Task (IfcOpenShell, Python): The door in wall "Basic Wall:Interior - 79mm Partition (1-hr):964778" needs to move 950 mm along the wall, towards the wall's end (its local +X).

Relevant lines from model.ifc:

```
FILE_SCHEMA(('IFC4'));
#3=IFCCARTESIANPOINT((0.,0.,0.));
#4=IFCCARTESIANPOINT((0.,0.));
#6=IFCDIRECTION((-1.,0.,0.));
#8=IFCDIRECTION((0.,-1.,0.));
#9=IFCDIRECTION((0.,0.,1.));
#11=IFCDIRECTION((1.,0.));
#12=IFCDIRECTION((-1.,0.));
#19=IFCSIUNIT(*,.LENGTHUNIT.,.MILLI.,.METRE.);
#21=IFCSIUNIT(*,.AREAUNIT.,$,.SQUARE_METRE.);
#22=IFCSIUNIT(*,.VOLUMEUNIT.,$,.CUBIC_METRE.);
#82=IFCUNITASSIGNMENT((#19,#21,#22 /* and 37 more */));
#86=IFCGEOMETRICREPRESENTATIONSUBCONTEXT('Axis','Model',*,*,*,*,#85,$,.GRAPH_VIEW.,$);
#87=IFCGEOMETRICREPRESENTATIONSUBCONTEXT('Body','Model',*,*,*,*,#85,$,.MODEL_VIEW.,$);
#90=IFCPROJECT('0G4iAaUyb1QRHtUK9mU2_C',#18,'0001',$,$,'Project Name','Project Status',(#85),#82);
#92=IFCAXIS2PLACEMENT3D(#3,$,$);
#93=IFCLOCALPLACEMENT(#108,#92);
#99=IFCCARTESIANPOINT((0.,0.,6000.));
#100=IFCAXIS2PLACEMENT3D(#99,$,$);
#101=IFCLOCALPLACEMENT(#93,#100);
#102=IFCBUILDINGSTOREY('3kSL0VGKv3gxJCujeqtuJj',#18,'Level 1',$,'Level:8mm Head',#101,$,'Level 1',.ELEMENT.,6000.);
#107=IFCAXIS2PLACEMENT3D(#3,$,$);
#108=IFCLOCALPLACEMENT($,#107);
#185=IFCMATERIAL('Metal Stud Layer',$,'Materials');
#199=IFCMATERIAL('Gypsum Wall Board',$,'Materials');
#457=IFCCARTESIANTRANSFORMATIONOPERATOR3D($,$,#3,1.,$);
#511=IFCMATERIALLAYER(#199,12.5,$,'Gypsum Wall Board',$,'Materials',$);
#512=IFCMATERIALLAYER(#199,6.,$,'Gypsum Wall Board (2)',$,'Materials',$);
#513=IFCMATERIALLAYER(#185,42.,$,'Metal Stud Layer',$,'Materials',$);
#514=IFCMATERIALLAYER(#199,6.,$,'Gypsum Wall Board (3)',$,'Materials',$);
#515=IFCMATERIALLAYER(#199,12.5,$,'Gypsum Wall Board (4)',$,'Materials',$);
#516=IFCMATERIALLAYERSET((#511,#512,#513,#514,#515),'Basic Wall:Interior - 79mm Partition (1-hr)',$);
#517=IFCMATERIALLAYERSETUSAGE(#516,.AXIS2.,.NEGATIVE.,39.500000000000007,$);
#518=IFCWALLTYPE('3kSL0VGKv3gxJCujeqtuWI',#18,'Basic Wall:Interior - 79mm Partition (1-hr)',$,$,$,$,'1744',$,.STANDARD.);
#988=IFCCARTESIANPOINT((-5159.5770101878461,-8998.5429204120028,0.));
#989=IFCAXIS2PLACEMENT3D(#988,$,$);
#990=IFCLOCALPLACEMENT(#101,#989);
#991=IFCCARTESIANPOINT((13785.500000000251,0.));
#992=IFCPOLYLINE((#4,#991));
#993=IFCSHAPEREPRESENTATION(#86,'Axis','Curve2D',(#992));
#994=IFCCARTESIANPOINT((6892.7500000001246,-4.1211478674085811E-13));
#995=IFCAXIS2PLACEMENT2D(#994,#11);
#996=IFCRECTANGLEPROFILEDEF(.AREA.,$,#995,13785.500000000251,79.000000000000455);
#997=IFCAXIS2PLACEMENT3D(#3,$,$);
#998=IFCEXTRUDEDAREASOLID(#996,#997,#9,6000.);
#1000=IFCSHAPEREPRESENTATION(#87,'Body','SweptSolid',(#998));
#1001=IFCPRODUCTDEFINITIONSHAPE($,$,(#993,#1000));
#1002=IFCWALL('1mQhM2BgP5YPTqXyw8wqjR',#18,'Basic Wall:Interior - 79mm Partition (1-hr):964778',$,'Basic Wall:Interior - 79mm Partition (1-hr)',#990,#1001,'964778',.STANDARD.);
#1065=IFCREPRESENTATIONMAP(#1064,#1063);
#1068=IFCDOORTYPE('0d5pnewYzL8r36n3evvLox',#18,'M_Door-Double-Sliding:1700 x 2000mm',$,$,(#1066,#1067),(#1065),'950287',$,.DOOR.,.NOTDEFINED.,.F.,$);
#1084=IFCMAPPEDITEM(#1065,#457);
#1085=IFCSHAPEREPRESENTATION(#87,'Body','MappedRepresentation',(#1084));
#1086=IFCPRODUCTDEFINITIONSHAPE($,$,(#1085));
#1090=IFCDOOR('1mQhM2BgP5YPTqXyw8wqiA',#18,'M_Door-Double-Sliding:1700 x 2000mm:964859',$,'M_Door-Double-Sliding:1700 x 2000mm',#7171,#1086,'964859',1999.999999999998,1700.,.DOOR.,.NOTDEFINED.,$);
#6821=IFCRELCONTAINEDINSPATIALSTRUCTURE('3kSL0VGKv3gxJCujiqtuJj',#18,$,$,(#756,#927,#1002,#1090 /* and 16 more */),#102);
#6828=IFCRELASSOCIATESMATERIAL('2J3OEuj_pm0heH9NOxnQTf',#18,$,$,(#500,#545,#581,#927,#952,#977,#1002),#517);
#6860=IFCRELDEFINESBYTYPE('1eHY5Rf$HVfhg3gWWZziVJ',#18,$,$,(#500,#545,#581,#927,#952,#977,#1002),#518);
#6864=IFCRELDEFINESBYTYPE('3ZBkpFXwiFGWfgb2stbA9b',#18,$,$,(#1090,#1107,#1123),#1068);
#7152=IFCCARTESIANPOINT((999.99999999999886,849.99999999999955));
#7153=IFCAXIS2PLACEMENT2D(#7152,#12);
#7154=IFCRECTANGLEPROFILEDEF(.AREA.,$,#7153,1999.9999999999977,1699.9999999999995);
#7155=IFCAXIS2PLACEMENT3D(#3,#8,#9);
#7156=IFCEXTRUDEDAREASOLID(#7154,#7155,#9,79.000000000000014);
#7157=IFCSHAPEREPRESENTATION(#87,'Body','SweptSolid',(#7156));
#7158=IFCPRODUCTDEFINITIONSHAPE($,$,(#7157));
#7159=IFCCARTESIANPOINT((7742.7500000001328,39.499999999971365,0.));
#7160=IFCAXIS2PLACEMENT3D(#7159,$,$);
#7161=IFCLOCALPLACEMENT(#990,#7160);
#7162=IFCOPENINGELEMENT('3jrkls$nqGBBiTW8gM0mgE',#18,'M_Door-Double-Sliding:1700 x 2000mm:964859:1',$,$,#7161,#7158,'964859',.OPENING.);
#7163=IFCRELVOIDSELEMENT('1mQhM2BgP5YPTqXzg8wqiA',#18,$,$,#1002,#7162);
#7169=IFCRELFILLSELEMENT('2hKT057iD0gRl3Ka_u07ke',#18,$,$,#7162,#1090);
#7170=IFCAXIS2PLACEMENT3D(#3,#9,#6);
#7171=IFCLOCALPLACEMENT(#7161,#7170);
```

```python
import ifcopenshell
import ifcopenshell.api.geometry
import ifcopenshell.util.placement

model = ifcopenshell.open("model.ifc")

door = model.by_guid("1mQhM2BgP5YPTqXyw8wqiA")
opening = door.FillsVoids[0].RelatingOpeningElement
wall = opening.VoidsElements[0].RelatingBuildingElement

wall_matrix = ifcopenshell.util.placement.get_local_placement(wall.ObjectPlacement)
shift = wall_matrix[:3, 0] * 950.0
before = ifcopenshell.util.placement.get_local_placement(door.ObjectPlacement)[:3, 3].copy()

# The door is placed relative to its opening, so it follows when the opening moves.
matrix = ifcopenshell.util.placement.get_local_placement(opening.ObjectPlacement)
matrix[:3, 3] += shift
ifcopenshell.api.geometry.edit_object_placement(
    model, product=opening, matrix=matrix, is_si=False, should_transform_children=True
)

after = ifcopenshell.util.placement.get_local_placement(door.ObjectPlacement)[:3, 3]
print("door moved by", (after - before).round(3) + 0.0)

model.write("model_v2.ifc")
```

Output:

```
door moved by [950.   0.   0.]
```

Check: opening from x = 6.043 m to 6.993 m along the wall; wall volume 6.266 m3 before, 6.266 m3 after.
